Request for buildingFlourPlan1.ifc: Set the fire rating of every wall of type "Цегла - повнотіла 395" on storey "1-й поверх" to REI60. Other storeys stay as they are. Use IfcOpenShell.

First a look at what the model holds.

```python
import ifcopenshell
import ifcopenshell.util.element

model = ifcopenshell.open("buildingFlourPlan1.ifc")
print(model.schema)
storey = next(s for s in model.by_type("IfcBuildingStorey") if s.Name == "1-й поверх")
walls = [e for e in ifcopenshell.util.element.get_decomposition(storey) if e.is_a("IfcWall")]
seen = {}
for e in walls:
    element_type = ifcopenshell.util.element.get_type(e)
    key = (element_type.Name if element_type != e and element_type else None, ifcopenshell.util.element.get_pset(e, "Pset_WallCommon", "FireRating"))
    seen[key] = seen.get(key, 0) + 1
for (name, value), count in sorted(seen.items(), key=str):
    print(count, "x", name, "|", value)
```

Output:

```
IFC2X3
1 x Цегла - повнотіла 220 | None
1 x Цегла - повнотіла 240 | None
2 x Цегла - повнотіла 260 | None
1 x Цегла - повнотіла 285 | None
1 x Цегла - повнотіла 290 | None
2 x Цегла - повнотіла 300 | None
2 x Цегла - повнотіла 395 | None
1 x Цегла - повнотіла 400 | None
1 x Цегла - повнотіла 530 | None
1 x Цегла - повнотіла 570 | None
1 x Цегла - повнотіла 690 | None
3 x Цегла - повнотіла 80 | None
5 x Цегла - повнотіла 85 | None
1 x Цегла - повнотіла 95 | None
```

```python
import ifcopenshell
import ifcopenshell.api.pset
import ifcopenshell.util.element

model = ifcopenshell.open("buildingFlourPlan1.ifc")

storey = next(s for s in model.by_type("IfcBuildingStorey") if s.Name == "1-й поверх")
walls = [e for e in ifcopenshell.util.element.get_decomposition(storey) if e.is_a("IfcWall")]

count = 0
for e in walls:
    element_type = ifcopenshell.util.element.get_type(e)
    if element_type in (None, e) or element_type.Name != "Цегла - повнотіла 395":
        continue
    # add_pset returns the element's existing set when there is one.
    pset = ifcopenshell.api.pset.add_pset(model, product=e, name="Pset_WallCommon")
    ifcopenshell.api.pset.edit_pset(model, pset=pset, properties={"FireRating": "REI60"})
    count += 1

print(count, "walls updated")

model.write("buildingFlourPlan1-out.ifc")
```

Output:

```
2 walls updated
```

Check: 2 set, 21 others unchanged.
